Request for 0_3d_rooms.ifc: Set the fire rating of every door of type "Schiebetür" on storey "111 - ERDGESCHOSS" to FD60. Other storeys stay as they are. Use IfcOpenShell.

First a look at what the model holds.

```python
import ifcopenshell
import ifcopenshell.util.element

model = ifcopenshell.open("0_3d_rooms.ifc")
print(model.schema)
storey = next(s for s in model.by_type("IfcBuildingStorey") if s.Name == "111 - ERDGESCHOSS")
doors = [e for e in ifcopenshell.util.element.get_decomposition(storey) if e.is_a("IfcDoor")]
seen = {}
for e in doors:
    element_type = ifcopenshell.util.element.get_type(e)
    key = (element_type.Name if element_type != e and element_type else None, ifcopenshell.util.element.get_pset(e, "Pset_DoorCommon", "FireRating"))
    seen[key] = seen.get(key, 0) + 1
for (name, value), count in sorted(seen.items(), key=str):
    print(count, "x", name, "|", value)
```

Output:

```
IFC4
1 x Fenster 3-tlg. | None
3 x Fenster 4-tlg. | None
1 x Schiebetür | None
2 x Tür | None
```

```python
import ifcopenshell
import ifcopenshell.api.pset
import ifcopenshell.util.element

model = ifcopenshell.open("0_3d_rooms.ifc")

storey = next(s for s in model.by_type("IfcBuildingStorey") if s.Name == "111 - ERDGESCHOSS")
doors = [e for e in ifcopenshell.util.element.get_decomposition(storey) if e.is_a("IfcDoor")]

count = 0
for e in doors:
    element_type = ifcopenshell.util.element.get_type(e)
    if element_type in (None, e) or element_type.Name != "Schiebetür":
        continue
    # add_pset returns the element's existing set when there is one.
    pset = ifcopenshell.api.pset.add_pset(model, product=e, name="Pset_DoorCommon")
    ifcopenshell.api.pset.edit_pset(model, pset=pset, properties={"FireRating": "FD60"})
    count += 1

print(count, "doors updated")

model.write("0_3d_rooms_edited.ifc")
```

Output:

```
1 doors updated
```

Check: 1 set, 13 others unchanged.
